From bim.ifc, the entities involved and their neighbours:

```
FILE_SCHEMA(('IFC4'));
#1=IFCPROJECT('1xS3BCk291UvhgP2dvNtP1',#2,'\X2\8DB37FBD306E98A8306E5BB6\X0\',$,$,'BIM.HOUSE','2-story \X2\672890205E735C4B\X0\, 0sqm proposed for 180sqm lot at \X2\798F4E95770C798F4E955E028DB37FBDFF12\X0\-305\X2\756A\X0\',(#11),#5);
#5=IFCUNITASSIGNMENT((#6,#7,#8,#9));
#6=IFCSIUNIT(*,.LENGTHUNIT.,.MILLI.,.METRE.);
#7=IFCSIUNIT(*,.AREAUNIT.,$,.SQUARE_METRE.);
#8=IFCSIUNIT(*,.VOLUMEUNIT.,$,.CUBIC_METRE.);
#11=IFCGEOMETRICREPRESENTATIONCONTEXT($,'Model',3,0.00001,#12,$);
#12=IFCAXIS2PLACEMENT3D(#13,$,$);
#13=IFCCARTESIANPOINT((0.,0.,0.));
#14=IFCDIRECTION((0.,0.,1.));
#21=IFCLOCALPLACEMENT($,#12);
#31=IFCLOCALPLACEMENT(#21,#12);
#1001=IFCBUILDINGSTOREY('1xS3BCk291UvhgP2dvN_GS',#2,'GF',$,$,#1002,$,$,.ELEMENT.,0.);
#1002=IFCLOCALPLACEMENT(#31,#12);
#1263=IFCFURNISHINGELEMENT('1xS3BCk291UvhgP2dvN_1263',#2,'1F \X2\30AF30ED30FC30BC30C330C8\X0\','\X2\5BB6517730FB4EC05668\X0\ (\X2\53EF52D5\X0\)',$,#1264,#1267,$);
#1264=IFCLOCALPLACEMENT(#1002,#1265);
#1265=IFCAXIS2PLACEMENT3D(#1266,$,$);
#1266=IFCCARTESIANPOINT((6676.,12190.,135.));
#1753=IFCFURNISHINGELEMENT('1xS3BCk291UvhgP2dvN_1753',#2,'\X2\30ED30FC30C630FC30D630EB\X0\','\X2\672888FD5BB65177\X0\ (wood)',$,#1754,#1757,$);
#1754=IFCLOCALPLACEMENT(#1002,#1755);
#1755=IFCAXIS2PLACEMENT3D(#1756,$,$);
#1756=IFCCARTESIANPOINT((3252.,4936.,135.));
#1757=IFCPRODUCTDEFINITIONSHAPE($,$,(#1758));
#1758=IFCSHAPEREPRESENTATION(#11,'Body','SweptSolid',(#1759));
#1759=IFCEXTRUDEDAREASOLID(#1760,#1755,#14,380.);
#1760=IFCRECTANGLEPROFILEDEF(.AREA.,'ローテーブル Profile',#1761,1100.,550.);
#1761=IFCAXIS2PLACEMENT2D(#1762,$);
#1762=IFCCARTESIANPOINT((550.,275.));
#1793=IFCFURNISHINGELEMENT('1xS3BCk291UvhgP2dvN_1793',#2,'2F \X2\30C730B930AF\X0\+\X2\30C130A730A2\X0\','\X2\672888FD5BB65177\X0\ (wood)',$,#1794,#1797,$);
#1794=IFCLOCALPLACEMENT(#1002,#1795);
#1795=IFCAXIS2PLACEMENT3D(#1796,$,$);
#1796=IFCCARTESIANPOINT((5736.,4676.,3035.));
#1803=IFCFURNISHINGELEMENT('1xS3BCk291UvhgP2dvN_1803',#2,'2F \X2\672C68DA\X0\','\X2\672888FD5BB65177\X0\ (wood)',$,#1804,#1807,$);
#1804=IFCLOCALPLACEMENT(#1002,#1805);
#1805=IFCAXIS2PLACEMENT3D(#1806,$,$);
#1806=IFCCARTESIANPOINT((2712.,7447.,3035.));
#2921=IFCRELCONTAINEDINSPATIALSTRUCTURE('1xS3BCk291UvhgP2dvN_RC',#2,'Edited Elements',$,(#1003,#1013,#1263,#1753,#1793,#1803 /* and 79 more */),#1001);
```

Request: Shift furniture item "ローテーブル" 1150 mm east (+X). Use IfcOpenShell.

```python
import ifcopenshell
import ifcopenshell.api.geometry
import ifcopenshell.util.placement
import ifcopenshell.util.unit

model = ifcopenshell.open("bim.ifc")
unit_scale = ifcopenshell.util.unit.calculate_unit_scale(model)

item = model.by_guid("1xS3BCk291UvhgP2dvN_1753")
matrix = ifcopenshell.util.placement.get_local_placement(item.ObjectPlacement)
matrix[0, 3] += 1.15 / unit_scale
ifcopenshell.api.geometry.edit_object_placement(model, product=item, matrix=matrix, is_si=False)

print(ifcopenshell.util.placement.get_local_placement(item.ObjectPlacement).round(3) + 0.0)

model.write("bim_rev.ifc")
```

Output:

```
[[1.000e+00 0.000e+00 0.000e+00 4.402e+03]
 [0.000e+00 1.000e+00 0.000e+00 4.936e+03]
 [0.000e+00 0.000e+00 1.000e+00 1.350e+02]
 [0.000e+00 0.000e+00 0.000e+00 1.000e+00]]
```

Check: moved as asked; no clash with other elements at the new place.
